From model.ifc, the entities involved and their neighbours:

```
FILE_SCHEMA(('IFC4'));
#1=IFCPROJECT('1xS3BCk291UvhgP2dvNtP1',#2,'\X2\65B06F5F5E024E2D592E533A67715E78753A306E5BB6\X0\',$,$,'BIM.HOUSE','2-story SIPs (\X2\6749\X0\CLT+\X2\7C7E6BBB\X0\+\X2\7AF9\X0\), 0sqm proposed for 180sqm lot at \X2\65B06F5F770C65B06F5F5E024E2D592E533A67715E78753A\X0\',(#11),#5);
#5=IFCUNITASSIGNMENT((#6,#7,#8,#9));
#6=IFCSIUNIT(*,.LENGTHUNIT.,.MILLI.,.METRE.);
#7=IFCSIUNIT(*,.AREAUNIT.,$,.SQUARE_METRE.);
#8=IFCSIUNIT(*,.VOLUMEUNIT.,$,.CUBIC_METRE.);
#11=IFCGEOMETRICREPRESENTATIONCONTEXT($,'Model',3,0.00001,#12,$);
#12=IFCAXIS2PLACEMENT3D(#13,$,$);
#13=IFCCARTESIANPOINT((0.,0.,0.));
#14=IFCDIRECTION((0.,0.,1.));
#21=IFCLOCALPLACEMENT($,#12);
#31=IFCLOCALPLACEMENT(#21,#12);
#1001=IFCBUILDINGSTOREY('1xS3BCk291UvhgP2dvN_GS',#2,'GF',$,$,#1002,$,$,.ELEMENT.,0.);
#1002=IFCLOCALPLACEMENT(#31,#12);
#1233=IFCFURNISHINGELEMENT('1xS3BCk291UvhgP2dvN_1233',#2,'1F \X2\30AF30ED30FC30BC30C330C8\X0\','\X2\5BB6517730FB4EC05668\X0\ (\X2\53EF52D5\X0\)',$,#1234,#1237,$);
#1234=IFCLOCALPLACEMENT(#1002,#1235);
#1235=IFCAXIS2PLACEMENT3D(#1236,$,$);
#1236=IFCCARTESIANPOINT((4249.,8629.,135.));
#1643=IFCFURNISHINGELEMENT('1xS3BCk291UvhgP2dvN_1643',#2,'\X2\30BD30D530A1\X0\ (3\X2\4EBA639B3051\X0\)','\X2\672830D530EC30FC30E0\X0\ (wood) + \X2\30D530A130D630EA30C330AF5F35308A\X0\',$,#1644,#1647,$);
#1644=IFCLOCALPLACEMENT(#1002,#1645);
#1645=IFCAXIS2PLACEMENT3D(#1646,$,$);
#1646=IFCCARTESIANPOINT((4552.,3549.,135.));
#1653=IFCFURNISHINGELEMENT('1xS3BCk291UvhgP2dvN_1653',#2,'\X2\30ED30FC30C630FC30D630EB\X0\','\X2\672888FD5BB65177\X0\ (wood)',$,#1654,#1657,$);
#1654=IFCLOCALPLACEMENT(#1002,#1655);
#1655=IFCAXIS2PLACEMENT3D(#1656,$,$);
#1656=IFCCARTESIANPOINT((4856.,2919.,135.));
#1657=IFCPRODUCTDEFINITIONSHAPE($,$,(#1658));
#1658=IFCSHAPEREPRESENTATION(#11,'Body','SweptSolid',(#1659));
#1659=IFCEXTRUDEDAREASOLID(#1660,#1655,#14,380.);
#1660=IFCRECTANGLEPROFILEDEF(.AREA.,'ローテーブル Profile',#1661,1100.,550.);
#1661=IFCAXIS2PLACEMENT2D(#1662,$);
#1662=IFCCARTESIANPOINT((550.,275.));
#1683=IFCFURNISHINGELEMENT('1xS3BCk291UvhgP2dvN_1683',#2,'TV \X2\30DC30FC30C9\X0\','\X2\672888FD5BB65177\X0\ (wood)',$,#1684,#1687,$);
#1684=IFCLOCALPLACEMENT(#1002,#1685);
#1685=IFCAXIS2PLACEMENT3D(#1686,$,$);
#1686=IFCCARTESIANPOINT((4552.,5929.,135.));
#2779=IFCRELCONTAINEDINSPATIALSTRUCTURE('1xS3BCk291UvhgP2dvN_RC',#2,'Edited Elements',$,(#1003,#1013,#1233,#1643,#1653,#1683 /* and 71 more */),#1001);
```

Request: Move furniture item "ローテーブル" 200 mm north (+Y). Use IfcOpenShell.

```python
import ifcopenshell
import ifcopenshell.api.geometry
import ifcopenshell.util.placement

model = ifcopenshell.open("model.ifc")

item = model.by_guid("1xS3BCk291UvhgP2dvN_1653")
matrix = ifcopenshell.util.placement.get_local_placement(item.ObjectPlacement)
matrix[1, 3] += 200.0
ifcopenshell.api.geometry.edit_object_placement(model, product=item, matrix=matrix, is_si=False)

print(ifcopenshell.util.placement.get_local_placement(item.ObjectPlacement).round(3) + 0.0)

model.write("model_rev.ifc")
```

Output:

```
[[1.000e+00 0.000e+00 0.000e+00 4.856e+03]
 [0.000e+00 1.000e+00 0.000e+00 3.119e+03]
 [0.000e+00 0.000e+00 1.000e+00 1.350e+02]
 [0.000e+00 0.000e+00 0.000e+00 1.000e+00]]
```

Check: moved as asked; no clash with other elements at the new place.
